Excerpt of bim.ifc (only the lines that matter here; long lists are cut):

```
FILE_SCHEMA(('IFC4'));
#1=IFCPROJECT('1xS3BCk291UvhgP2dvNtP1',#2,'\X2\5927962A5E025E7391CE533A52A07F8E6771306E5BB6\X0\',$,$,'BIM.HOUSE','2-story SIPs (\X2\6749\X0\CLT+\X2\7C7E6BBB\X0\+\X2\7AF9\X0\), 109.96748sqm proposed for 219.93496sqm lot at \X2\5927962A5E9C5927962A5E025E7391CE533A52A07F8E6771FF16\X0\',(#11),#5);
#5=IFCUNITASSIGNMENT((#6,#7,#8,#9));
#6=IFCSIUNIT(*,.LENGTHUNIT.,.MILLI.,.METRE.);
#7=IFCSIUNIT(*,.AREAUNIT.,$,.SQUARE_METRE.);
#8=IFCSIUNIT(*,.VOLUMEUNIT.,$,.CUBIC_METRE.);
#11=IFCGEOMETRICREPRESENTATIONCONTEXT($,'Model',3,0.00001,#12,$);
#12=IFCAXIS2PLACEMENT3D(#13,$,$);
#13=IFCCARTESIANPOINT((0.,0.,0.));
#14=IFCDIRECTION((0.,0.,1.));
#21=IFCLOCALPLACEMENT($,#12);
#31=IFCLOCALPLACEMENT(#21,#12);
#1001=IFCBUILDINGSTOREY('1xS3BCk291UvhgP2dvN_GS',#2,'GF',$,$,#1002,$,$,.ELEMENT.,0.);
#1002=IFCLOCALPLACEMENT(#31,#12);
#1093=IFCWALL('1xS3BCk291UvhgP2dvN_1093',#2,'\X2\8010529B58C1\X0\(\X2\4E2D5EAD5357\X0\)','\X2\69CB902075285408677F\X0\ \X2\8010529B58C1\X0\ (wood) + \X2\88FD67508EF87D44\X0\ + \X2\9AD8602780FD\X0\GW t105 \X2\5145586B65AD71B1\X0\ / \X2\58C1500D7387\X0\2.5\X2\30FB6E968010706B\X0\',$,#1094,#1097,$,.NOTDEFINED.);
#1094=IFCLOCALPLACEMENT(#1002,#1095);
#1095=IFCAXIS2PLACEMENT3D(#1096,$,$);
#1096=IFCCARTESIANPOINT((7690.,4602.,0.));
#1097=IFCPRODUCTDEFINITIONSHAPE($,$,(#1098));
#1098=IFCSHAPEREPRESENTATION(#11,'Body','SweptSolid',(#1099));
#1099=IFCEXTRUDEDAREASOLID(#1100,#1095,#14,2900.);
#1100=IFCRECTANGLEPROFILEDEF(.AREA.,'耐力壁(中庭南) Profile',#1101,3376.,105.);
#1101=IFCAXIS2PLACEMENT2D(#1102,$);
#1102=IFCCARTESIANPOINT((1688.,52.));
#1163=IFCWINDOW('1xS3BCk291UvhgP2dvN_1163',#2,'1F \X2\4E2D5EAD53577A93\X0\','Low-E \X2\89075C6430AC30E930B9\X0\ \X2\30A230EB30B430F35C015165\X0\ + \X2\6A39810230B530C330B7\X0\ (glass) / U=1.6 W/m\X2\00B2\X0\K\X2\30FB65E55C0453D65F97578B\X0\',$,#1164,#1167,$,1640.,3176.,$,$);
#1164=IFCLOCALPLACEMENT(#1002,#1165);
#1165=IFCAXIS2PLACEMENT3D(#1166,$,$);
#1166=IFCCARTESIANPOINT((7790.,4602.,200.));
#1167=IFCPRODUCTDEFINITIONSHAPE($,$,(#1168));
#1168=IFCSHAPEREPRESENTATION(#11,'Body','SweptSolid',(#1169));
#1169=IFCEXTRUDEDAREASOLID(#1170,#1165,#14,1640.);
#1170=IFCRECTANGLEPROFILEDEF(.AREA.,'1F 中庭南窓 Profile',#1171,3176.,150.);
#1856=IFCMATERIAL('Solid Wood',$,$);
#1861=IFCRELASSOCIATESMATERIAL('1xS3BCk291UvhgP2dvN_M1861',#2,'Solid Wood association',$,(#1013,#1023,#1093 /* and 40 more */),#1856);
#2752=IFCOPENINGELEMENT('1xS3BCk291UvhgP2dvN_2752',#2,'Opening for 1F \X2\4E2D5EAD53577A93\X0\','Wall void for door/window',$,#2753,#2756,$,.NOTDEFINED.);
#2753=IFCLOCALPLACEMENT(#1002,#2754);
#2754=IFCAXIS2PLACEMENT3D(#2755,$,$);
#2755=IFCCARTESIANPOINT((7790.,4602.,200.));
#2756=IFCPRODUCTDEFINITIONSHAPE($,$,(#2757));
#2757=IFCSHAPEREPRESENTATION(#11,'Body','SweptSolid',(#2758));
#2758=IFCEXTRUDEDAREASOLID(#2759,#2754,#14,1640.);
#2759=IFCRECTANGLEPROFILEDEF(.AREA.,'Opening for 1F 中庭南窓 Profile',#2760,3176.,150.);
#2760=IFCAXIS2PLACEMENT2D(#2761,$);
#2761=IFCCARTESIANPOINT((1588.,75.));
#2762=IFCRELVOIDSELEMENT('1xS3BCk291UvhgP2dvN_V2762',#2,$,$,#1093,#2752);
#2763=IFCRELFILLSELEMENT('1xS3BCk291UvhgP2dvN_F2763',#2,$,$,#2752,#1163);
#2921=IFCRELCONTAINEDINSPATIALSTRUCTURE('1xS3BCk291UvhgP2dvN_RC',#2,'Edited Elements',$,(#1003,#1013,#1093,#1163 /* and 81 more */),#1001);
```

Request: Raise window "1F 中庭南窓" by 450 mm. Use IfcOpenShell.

```python
import numpy as np
import ifcopenshell
import ifcopenshell.api.geometry
import ifcopenshell.util.placement
import ifcopenshell.util.unit

model = ifcopenshell.open("bim.ifc")
unit_scale = ifcopenshell.util.unit.calculate_unit_scale(model)

window = model.by_guid("1xS3BCk291UvhgP2dvN_1163")
opening = window.FillsVoids[0].RelatingOpeningElement
dz = 450.0

shift = np.array([0.0, 0.0, dz])
# The window is not placed relative to its opening, so move both.
for product in (opening, window):
    matrix = ifcopenshell.util.placement.get_local_placement(product.ObjectPlacement)
    matrix[:3, 3] += shift
    ifcopenshell.api.geometry.edit_object_placement(model, product=product, matrix=matrix, is_si=False)

print(f"moved by {dz * unit_scale:+.3f} m")

model.write("bim_updated.ifc")
```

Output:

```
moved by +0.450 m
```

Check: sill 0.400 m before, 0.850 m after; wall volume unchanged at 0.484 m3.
